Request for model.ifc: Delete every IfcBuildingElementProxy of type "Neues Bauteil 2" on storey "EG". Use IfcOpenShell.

First a look at what the model holds.

```python
import ifcopenshell
import ifcopenshell.util.element

model = ifcopenshell.open("model.ifc")
print(model.schema)
storey = next(s for s in model.by_type("IfcBuildingStorey") if s.Name == "EG")
proxies = [e for e in ifcopenshell.util.element.get_decomposition(storey) if e.is_a("IfcBuildingElementProxy")]
seen = {}
for e in proxies:
    element_type = ifcopenshell.util.element.get_type(e)
    name = element_type.Name if element_type not in (None, e) else None
    seen[name] = seen.get(name, 0) + 1
for name, count in sorted(seen.items(), key=str):
    print(count, "x", name)
```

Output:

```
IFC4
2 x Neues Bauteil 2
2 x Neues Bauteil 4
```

```python
import ifcopenshell
import ifcopenshell.api.root
import ifcopenshell.util.element

model = ifcopenshell.open("model.ifc")

storey = next(s for s in model.by_type("IfcBuildingStorey") if s.Name == "EG")
proxies = [e for e in ifcopenshell.util.element.get_decomposition(storey) if e.is_a("IfcBuildingElementProxy")]
targets = [e for e in proxies if (t := ifcopenshell.util.element.get_type(e)) not in (None, e) and t.Name == "Neues Bauteil 2"]

for e in targets:
    ifcopenshell.api.root.remove_product(model, product=e)
print(len(targets), "removed")

model.write("model-out.ifc")
```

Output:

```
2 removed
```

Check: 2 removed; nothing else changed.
